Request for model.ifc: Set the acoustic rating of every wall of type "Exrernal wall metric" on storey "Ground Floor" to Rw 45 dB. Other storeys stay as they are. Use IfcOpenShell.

First a look at what the model holds.

```python
import ifcopenshell
import ifcopenshell.util.element

model = ifcopenshell.open("model.ifc")
print(model.schema)
storey = next(s for s in model.by_type("IfcBuildingStorey") if s.Name == "Ground Floor")
walls = [e for e in ifcopenshell.util.element.get_decomposition(storey) if e.is_a("IfcWall")]
seen = {}
for e in walls:
    element_type = ifcopenshell.util.element.get_type(e)
    key = (element_type.Name if element_type != e and element_type else None, ifcopenshell.util.element.get_pset(e, "Pset_WallCommon", "AcousticRating"))
    seen[key] = seen.get(key, 0) + 1
for (name, value), count in sorted(seen.items(), key=str):
    print(count, "x", name, "|", value)
```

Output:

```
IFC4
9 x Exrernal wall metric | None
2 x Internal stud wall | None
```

```python
import ifcopenshell
import ifcopenshell.api.pset
import ifcopenshell.util.element

model = ifcopenshell.open("model.ifc")

storey = next(s for s in model.by_type("IfcBuildingStorey") if s.Name == "Ground Floor")
walls = [e for e in ifcopenshell.util.element.get_decomposition(storey) if e.is_a("IfcWall")]

count = 0
for e in walls:
    element_type = ifcopenshell.util.element.get_type(e)
    if element_type in (None, e) or element_type.Name != "Exrernal wall metric":
        continue
    # add_pset returns the element's existing set when there is one.
    pset = ifcopenshell.api.pset.add_pset(model, product=e, name="Pset_WallCommon")
    ifcopenshell.api.pset.edit_pset(model, pset=pset, properties={"AcousticRating": "Rw 45 dB"})
    count += 1

print(count, "walls updated")

model.write("model_rev.ifc")
```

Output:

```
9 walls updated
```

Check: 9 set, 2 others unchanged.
